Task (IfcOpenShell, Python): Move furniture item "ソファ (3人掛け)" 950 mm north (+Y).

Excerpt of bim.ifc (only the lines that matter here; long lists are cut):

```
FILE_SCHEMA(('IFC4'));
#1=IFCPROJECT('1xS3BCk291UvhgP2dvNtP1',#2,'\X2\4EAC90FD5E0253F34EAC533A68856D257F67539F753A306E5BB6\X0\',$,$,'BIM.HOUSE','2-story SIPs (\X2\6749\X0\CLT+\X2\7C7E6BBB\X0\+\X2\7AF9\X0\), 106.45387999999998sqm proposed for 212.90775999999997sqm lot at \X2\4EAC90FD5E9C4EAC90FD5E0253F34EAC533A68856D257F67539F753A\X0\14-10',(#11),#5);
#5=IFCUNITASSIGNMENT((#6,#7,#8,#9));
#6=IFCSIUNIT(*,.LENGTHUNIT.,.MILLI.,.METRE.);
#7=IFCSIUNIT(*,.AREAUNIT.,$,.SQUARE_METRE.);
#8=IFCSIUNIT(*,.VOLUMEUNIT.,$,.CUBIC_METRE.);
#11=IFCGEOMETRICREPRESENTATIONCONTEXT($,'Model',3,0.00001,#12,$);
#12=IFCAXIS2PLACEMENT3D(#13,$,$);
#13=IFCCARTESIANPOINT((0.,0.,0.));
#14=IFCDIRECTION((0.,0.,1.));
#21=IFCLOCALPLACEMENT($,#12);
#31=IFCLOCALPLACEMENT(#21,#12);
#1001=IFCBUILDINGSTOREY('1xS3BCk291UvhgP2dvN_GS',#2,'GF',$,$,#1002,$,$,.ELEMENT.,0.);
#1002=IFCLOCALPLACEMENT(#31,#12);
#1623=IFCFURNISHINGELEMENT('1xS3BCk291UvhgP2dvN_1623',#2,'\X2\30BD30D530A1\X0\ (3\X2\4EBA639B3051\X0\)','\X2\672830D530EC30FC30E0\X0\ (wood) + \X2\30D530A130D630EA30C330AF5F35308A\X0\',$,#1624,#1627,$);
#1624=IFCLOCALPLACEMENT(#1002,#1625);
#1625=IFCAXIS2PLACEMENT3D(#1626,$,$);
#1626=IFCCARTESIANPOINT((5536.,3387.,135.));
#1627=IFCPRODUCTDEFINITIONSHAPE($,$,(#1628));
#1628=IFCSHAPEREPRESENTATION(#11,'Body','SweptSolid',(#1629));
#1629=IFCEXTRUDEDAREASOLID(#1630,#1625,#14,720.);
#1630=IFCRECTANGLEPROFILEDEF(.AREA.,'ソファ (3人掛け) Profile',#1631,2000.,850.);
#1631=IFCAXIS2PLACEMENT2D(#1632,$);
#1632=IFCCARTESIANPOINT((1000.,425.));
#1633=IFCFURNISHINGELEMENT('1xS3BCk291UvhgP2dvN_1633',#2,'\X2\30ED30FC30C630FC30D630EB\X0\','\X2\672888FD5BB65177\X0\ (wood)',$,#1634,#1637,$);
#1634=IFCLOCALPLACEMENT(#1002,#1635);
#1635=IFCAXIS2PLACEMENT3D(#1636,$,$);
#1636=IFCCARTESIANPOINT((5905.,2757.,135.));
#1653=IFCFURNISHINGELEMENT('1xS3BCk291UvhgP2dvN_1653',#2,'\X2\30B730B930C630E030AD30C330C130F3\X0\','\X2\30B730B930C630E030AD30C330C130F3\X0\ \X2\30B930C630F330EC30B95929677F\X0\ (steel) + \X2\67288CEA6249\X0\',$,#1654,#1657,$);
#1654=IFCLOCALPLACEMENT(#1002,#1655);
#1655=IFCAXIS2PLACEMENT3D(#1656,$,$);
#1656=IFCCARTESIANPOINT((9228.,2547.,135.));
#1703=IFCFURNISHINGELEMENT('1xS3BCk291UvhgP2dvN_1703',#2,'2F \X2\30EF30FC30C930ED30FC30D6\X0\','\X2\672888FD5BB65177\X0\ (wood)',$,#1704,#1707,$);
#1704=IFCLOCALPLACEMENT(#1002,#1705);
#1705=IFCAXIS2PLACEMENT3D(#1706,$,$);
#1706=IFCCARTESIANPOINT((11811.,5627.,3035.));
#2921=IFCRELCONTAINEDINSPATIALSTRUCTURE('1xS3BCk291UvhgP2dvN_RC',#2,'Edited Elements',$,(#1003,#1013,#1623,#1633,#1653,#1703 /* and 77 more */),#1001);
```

```python
import ifcopenshell
import ifcopenshell.api.geometry
import ifcopenshell.util.placement
import ifcopenshell.util.unit

model = ifcopenshell.open("bim.ifc")
unit_scale = ifcopenshell.util.unit.calculate_unit_scale(model)

item = model.by_guid("1xS3BCk291UvhgP2dvN_1623")
matrix = ifcopenshell.util.placement.get_local_placement(item.ObjectPlacement)
matrix[1, 3] += 0.95 / unit_scale
ifcopenshell.api.geometry.edit_object_placement(model, product=item, matrix=matrix, is_si=False)

print(ifcopenshell.util.placement.get_local_placement(item.ObjectPlacement).round(3) + 0.0)

model.write("bim_edited.ifc")
```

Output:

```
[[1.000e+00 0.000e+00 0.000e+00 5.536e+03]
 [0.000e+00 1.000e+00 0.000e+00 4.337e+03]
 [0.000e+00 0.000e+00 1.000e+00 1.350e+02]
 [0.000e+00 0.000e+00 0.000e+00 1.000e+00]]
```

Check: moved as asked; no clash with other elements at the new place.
